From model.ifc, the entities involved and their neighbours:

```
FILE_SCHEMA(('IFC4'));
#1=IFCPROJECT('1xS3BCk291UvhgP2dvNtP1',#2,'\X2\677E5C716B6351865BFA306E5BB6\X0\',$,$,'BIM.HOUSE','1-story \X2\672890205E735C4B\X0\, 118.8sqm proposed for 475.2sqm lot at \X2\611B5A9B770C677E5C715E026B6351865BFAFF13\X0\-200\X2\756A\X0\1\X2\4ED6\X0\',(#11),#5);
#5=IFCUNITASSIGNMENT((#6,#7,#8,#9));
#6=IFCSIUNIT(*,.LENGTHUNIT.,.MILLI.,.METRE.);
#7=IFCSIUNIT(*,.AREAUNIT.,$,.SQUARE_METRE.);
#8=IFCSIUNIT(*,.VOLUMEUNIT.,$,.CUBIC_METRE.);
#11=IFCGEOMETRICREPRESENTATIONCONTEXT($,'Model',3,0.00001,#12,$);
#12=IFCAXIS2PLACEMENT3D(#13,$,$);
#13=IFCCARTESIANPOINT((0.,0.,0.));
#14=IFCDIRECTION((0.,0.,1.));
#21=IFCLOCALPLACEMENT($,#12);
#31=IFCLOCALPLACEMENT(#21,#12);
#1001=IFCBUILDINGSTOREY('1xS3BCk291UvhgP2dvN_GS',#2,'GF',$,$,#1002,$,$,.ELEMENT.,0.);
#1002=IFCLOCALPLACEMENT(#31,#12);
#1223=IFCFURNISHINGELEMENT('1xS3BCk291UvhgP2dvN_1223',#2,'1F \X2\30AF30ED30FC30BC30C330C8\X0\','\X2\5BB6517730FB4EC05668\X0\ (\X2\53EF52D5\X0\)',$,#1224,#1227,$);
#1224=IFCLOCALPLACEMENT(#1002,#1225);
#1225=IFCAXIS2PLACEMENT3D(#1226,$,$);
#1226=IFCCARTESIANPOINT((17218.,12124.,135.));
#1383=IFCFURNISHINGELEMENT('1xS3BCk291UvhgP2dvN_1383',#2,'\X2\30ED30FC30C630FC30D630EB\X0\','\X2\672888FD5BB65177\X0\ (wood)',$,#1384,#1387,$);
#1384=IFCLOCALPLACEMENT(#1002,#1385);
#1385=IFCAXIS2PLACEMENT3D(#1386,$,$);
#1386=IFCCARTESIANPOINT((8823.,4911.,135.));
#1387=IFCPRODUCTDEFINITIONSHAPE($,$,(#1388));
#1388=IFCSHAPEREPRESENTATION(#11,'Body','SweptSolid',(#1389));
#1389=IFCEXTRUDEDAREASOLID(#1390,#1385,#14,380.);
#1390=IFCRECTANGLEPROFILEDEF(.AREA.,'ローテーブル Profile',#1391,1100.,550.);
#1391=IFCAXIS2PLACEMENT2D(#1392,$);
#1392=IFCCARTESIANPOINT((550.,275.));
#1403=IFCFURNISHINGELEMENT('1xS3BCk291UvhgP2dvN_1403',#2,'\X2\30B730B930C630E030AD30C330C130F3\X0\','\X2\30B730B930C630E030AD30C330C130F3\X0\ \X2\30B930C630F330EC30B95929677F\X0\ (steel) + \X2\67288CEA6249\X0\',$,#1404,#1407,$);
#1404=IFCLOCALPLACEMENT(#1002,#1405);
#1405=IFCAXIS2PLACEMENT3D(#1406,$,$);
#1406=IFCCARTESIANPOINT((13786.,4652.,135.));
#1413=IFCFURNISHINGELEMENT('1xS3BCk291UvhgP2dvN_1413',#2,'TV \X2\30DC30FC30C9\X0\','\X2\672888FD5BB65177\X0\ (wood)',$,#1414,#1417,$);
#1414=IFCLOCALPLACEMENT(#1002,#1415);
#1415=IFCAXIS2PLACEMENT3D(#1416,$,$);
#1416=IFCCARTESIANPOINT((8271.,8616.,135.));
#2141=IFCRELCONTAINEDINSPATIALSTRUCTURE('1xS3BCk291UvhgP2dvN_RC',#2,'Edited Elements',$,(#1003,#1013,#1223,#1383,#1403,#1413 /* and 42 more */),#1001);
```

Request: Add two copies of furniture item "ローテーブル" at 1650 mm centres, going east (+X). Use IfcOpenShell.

```python
import numpy as np
import ifcopenshell
import ifcopenshell.api.geometry
import ifcopenshell.api.root
import ifcopenshell.util.element
import ifcopenshell.util.placement
import ifcopenshell.util.unit

model = ifcopenshell.open("model.ifc")
unit_scale = ifcopenshell.util.unit.calculate_unit_scale(model)


def reuse_history(source, copy):
    """copy_class also copies each property set's owner history, people and application; keep the originals."""
    for rel in copy.IsDefinedBy:
        if rel.is_a("IfcRelDefinesByProperties") and (history := rel.RelatingPropertyDefinition.OwnerHistory):
            rel.RelatingPropertyDefinition.OwnerHistory = source.OwnerHistory
            ifcopenshell.util.element.remove_deep2(model, history)


source = model.by_guid("1xS3BCk291UvhgP2dvN_1383")
base = ifcopenshell.util.placement.get_local_placement(source.ObjectPlacement)
step = np.array([1.0, 0.0, 0.0]) * 1.65 / unit_scale

for i in range(1, 3):
    copy = ifcopenshell.api.root.copy_class(model, product=source)
    copy.Representation = ifcopenshell.util.element.copy_deep(
        model, source.Representation, exclude=["IfcGeometricRepresentationContext", "IfcRepresentationMap"]
    )
    reuse_history(source, copy)
    matrix = base.copy()
    matrix[:3, 3] += i * step
    print("added at", matrix[:3, 3].round(3) + 0.0)
    ifcopenshell.api.geometry.edit_object_placement(model, product=copy, matrix=matrix, is_si=False)

model.write("model_rev.ifc")
```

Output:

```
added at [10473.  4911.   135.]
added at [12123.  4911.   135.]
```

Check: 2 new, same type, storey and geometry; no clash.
